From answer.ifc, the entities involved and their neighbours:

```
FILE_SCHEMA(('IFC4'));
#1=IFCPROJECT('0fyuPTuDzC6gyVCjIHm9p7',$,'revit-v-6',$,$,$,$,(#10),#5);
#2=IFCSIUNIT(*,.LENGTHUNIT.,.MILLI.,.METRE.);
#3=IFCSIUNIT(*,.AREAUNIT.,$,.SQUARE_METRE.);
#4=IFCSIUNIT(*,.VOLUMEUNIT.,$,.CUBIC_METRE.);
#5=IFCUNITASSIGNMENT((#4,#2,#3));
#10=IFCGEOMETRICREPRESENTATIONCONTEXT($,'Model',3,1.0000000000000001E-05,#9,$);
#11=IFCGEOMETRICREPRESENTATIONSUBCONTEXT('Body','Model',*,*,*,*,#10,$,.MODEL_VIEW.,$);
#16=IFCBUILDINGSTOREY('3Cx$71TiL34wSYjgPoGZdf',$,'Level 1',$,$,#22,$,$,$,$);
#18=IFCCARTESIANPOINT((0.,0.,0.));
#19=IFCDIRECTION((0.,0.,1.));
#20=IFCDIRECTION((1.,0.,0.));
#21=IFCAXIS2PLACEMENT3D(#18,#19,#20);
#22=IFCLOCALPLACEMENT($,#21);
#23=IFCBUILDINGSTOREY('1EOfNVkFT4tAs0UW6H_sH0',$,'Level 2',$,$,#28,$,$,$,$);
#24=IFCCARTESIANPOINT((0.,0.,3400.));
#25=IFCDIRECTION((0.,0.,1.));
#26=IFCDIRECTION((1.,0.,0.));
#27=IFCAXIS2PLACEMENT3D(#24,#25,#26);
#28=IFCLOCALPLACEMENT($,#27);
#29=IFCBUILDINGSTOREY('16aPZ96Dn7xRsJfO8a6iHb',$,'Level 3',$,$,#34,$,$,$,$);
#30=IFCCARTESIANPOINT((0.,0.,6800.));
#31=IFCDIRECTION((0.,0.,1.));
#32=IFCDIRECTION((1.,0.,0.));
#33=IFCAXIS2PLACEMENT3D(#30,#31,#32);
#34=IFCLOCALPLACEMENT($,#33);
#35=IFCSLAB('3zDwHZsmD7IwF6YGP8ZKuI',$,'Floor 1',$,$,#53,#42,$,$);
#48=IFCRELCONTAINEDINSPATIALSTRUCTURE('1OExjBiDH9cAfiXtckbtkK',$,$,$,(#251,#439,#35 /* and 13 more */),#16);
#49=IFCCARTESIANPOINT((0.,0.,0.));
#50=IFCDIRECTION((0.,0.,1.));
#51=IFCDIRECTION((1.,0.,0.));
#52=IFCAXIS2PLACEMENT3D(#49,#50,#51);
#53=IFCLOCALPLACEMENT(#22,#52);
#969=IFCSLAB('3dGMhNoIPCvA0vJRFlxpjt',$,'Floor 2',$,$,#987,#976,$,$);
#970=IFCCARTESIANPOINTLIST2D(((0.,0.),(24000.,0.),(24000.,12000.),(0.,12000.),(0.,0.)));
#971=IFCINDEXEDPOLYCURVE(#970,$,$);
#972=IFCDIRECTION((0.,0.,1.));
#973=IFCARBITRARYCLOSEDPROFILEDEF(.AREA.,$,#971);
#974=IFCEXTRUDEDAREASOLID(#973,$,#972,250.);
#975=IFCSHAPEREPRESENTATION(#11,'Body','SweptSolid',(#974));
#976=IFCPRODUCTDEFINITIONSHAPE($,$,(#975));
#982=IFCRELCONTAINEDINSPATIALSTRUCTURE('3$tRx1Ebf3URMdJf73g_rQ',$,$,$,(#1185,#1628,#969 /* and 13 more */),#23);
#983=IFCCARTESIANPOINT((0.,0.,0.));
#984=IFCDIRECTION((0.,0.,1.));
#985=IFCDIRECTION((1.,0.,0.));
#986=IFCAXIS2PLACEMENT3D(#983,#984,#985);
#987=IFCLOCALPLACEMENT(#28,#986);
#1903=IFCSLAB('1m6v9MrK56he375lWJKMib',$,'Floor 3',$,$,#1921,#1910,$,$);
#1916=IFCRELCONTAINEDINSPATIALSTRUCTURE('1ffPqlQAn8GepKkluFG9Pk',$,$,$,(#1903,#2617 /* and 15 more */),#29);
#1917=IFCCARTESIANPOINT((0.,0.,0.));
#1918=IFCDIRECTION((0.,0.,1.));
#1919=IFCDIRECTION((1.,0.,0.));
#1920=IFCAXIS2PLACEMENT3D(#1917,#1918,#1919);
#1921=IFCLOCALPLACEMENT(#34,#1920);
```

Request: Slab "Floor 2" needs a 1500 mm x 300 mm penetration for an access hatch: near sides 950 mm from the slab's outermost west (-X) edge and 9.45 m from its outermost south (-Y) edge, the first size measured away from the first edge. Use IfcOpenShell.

```python
import numpy as np
import ifcopenshell
import ifcopenshell.api.feature
import ifcopenshell.api.geometry
import ifcopenshell.api.root
import ifcopenshell.geom
import ifcopenshell.util.placement
import ifcopenshell.util.representation
import ifcopenshell.util.shape
import ifcopenshell.util.unit

model = ifcopenshell.open("answer.ifc")
unit_scale = ifcopenshell.util.unit.calculate_unit_scale(model)
settings = ifcopenshell.geom.settings()


def volume(element):
    """Net volume in cubic metres, openings subtracted."""
    shape = ifcopenshell.geom.create_shape(settings, element)
    return ifcopenshell.util.shape.get_volume(shape.geometry)


slab = model.by_guid("3dGMhNoIPCvA0vJRFlxpjt")
before = volume(slab)

# Extent in the slab's own axes, in metres. The edges named are its -X and -Y sides.
slab_shape = ifcopenshell.geom.create_shape(settings, slab)
vertices = ifcopenshell.util.shape.get_vertices(slab_shape.geometry)
x_min, y_min, bottom = vertices.min(axis=0)
top = vertices[:, 2].max()

opening = ifcopenshell.api.root.create_entity(model, ifc_class="IfcOpeningElement", name="Access hatch opening", predefined_type="OPENING")
context = ifcopenshell.util.representation.get_context(model, "Model", "Body", "MODEL_VIEW")
width, depth = 1.5, 0.3
outline = [(0.0, 0.0), (width, 0.0), (width, depth), (0.0, depth), (0.0, 0.0)]
# Overshoot both faces by 50 mm so the cut is clean.
shape = ifcopenshell.api.geometry.add_slab_representation(
    model, context=context, depth=top - bottom + 0.1, polyline=outline
)
ifcopenshell.api.geometry.assign_representation(model, product=opening, representation=shape)

matrix = ifcopenshell.util.placement.get_local_placement(slab.ObjectPlacement)
matrix[:, 3] = matrix @ np.append(np.array([x_min + 0.95, y_min + 9.45, bottom - 0.05]) / unit_scale, 1.0)
ifcopenshell.api.geometry.edit_object_placement(model, product=opening, matrix=matrix, is_si=False)
ifcopenshell.api.feature.add_feature(model, feature=opening, element=slab)

after = volume(slab)

print(f"slab volume {before:.3f} -> {after:.3f} m3")

model.write("answer_v2.ifc")
```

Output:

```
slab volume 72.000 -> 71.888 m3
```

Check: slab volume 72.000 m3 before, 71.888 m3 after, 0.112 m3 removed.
